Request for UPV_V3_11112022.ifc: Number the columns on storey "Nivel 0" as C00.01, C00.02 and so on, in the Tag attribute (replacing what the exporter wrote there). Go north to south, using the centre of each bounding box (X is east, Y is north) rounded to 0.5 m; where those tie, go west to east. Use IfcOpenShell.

First a look at what the model holds.

```python
import ifcopenshell
import ifcopenshell.util.element
import ifcopenshell.util.placement

model = ifcopenshell.open("UPV_V3_11112022.ifc")
print(model.schema)
storey = next(s for s in model.by_type("IfcBuildingStorey") if s.Name == "Nivel 0")
columns = [e for e in ifcopenshell.util.element.get_decomposition(storey) if e.is_a("IfcColumn")]
for e in sorted(columns, key=lambda e: e.id()):
    origin = ifcopenshell.util.placement.get_local_placement(e.ObjectPlacement)[:3, 3]
    print(e.id(), e.Tag, e.Name, origin.round(2) + 0.0, sep=" | ")
```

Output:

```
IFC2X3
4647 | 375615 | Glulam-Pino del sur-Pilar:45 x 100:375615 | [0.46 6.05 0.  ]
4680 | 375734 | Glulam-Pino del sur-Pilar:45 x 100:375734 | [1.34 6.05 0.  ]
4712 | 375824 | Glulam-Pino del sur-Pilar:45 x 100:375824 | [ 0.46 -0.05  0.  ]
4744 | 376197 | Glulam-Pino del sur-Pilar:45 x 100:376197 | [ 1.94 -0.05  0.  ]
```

```python
import ifcopenshell
import ifcopenshell.geom
import ifcopenshell.util.element
import ifcopenshell.util.shape

model = ifcopenshell.open("UPV_V3_11112022.ifc")
settings = ifcopenshell.geom.settings()
settings.set("use-world-coords", True)


def centre(element):
    shape = ifcopenshell.geom.create_shape(settings, element)
    return ifcopenshell.util.shape.get_bbox_centroid(shape.geometry)


storey = next(s for s in model.by_type("IfcBuildingStorey") if s.Name == "Nivel 0")
columns = [e for e in ifcopenshell.util.element.get_decomposition(storey) if e.is_a("IfcColumn")]

# Insertion points can sit at a corner or the storey origin, so sort by the geometry (in metres).
centres = {e: centre(e) for e in columns}
columns.sort(key=lambda e: (-round(centres[e][1] / 0.5), centres[e][0]))

for i, e in enumerate(columns, start=1):
    number = f"C00.{i:02d}"
    e.Tag = number
    print(e.id(), number)

model.write("UPV_V3_11112022-out.ifc")
```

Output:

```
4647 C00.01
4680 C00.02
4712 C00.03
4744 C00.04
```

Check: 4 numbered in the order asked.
